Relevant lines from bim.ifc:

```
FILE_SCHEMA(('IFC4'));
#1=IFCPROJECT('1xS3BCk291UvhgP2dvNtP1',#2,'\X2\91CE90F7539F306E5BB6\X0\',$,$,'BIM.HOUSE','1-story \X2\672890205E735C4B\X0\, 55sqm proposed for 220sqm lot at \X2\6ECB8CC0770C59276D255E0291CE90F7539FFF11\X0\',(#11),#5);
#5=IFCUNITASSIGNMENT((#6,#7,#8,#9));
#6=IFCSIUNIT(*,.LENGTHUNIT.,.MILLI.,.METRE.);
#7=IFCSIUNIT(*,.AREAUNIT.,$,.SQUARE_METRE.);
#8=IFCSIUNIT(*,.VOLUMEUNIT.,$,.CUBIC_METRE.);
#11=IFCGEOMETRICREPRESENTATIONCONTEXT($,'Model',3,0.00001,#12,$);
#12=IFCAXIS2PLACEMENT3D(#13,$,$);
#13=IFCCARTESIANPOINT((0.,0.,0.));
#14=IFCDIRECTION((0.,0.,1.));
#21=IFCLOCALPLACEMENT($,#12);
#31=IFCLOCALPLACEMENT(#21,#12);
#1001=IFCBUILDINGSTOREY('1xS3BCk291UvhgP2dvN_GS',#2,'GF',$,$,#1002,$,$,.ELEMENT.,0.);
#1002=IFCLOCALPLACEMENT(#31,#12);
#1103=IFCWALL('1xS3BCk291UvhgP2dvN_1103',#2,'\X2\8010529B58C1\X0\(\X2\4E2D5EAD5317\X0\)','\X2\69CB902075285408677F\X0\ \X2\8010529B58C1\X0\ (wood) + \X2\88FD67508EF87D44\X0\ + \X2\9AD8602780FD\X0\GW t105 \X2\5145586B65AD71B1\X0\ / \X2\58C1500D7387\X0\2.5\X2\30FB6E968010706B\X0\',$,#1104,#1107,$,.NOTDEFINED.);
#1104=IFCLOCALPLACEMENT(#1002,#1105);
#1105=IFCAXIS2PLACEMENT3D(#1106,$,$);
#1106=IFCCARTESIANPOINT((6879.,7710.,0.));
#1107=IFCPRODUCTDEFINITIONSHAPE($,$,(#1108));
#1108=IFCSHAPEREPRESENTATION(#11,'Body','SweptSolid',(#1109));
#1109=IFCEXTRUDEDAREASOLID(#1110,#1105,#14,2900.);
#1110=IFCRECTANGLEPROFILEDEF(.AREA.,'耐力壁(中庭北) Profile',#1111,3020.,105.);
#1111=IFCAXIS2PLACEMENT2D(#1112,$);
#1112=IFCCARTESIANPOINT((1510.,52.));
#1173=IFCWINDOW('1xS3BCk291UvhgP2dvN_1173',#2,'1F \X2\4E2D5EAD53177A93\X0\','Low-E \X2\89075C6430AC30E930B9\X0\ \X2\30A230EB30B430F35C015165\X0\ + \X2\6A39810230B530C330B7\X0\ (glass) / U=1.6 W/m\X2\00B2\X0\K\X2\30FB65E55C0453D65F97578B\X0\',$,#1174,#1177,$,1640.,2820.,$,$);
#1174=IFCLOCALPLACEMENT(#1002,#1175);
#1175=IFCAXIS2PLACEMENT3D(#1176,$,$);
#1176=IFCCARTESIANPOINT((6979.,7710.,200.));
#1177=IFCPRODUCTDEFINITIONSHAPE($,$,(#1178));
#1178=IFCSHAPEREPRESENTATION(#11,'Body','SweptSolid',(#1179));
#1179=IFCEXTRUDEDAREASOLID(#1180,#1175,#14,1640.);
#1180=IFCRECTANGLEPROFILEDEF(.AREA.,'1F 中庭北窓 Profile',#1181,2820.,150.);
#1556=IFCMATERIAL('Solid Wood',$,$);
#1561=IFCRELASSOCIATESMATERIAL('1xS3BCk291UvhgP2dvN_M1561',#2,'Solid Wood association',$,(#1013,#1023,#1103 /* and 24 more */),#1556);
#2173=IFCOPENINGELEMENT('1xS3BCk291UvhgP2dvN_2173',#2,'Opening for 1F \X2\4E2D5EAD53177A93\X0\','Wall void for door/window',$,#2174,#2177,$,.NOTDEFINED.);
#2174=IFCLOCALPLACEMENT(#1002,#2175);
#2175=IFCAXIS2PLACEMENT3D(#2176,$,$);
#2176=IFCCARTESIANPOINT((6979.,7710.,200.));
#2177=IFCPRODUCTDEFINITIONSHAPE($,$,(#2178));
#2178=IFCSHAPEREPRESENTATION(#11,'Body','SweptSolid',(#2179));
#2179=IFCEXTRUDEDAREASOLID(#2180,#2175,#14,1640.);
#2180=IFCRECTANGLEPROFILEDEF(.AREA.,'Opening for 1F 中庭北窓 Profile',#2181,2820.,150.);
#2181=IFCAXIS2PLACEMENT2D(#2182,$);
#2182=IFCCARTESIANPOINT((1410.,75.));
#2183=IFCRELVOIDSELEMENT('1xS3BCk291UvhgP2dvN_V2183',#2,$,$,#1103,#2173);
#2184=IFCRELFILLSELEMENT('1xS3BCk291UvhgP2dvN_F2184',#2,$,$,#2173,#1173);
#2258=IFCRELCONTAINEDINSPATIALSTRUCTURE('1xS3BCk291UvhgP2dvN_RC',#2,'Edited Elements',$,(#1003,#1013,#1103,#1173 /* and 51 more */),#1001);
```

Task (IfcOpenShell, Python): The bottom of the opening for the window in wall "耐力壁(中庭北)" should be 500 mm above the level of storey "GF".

```python
import numpy as np
import ifcopenshell
import ifcopenshell.api.geometry
import ifcopenshell.geom
import ifcopenshell.util.element
import ifcopenshell.util.placement
import ifcopenshell.util.shape
import ifcopenshell.util.unit

model = ifcopenshell.open("bim.ifc")
unit_scale = ifcopenshell.util.unit.calculate_unit_scale(model)

window = model.by_guid("1xS3BCk291UvhgP2dvN_1173")
opening = window.FillsVoids[0].RelatingOpeningElement
storey = ifcopenshell.util.element.get_container(window, ifc_class="IfcBuildingStorey")
level = ifcopenshell.util.placement.get_local_placement(storey.ObjectPlacement)[2, 3]

# The opening's origin need not be at the sill, so measure its lowest point.
shape = ifcopenshell.geom.create_shape(ifcopenshell.geom.settings(), opening)
bottom = ifcopenshell.util.shape.get_shape_bottom_elevation(shape, shape.geometry) / unit_scale
dz = level + 0.5 / unit_scale - bottom

shift = np.array([0.0, 0.0, dz])
# The window is not placed relative to its opening, so move both.
for product in (opening, window):
    matrix = ifcopenshell.util.placement.get_local_placement(product.ObjectPlacement)
    matrix[:3, 3] += shift
    ifcopenshell.api.geometry.edit_object_placement(model, product=product, matrix=matrix, is_si=False)

print(f"moved by {dz * unit_scale:+.3f} m")

model.write("bim_v2.ifc")
```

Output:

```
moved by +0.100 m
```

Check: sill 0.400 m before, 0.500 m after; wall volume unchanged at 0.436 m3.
